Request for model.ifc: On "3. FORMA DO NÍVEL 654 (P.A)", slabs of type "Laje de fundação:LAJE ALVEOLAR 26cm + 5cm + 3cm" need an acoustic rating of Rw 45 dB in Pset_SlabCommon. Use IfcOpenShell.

First a look at what the model holds.

```python
import ifcopenshell
import ifcopenshell.util.element

model = ifcopenshell.open("model.ifc")
print(model.schema)
storey = next(s for s in model.by_type("IfcBuildingStorey") if s.Name == "3. FORMA DO NÍVEL 654 (P.A)")
slabs = [e for e in ifcopenshell.util.element.get_decomposition(storey) if e.is_a("IfcSlab")]
seen = {}
for e in slabs:
    element_type = ifcopenshell.util.element.get_type(e)
    key = (element_type.Name if element_type != e and element_type else None, ifcopenshell.util.element.get_pset(e, "Pset_SlabCommon", "AcousticRating"))
    seen[key] = seen.get(key, 0) + 1
for (name, value), count in sorted(seen.items(), key=str):
    print(count, "x", name, "|", value)
```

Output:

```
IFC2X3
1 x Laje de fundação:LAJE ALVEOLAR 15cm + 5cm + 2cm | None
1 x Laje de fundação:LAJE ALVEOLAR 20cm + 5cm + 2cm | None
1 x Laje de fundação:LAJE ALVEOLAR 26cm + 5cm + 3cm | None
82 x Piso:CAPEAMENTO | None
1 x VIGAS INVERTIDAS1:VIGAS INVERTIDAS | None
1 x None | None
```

```python
import ifcopenshell
import ifcopenshell.api.pset
import ifcopenshell.util.element

model = ifcopenshell.open("model.ifc")

storey = next(s for s in model.by_type("IfcBuildingStorey") if s.Name == "3. FORMA DO NÍVEL 654 (P.A)")
slabs = [e for e in ifcopenshell.util.element.get_decomposition(storey) if e.is_a("IfcSlab")]

count = 0
for e in slabs:
    element_type = ifcopenshell.util.element.get_type(e)
    if element_type in (None, e) or element_type.Name != "Laje de fundação:LAJE ALVEOLAR 26cm + 5cm + 3cm":
        continue
    # add_pset returns the element's existing set when there is one.
    pset = ifcopenshell.api.pset.add_pset(model, product=e, name="Pset_SlabCommon")
    ifcopenshell.api.pset.edit_pset(model, pset=pset, properties={"AcousticRating": "Rw 45 dB"})
    count += 1

print(count, "slabs updated")

model.write("model_edited.ifc")
```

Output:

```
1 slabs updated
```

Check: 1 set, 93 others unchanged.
